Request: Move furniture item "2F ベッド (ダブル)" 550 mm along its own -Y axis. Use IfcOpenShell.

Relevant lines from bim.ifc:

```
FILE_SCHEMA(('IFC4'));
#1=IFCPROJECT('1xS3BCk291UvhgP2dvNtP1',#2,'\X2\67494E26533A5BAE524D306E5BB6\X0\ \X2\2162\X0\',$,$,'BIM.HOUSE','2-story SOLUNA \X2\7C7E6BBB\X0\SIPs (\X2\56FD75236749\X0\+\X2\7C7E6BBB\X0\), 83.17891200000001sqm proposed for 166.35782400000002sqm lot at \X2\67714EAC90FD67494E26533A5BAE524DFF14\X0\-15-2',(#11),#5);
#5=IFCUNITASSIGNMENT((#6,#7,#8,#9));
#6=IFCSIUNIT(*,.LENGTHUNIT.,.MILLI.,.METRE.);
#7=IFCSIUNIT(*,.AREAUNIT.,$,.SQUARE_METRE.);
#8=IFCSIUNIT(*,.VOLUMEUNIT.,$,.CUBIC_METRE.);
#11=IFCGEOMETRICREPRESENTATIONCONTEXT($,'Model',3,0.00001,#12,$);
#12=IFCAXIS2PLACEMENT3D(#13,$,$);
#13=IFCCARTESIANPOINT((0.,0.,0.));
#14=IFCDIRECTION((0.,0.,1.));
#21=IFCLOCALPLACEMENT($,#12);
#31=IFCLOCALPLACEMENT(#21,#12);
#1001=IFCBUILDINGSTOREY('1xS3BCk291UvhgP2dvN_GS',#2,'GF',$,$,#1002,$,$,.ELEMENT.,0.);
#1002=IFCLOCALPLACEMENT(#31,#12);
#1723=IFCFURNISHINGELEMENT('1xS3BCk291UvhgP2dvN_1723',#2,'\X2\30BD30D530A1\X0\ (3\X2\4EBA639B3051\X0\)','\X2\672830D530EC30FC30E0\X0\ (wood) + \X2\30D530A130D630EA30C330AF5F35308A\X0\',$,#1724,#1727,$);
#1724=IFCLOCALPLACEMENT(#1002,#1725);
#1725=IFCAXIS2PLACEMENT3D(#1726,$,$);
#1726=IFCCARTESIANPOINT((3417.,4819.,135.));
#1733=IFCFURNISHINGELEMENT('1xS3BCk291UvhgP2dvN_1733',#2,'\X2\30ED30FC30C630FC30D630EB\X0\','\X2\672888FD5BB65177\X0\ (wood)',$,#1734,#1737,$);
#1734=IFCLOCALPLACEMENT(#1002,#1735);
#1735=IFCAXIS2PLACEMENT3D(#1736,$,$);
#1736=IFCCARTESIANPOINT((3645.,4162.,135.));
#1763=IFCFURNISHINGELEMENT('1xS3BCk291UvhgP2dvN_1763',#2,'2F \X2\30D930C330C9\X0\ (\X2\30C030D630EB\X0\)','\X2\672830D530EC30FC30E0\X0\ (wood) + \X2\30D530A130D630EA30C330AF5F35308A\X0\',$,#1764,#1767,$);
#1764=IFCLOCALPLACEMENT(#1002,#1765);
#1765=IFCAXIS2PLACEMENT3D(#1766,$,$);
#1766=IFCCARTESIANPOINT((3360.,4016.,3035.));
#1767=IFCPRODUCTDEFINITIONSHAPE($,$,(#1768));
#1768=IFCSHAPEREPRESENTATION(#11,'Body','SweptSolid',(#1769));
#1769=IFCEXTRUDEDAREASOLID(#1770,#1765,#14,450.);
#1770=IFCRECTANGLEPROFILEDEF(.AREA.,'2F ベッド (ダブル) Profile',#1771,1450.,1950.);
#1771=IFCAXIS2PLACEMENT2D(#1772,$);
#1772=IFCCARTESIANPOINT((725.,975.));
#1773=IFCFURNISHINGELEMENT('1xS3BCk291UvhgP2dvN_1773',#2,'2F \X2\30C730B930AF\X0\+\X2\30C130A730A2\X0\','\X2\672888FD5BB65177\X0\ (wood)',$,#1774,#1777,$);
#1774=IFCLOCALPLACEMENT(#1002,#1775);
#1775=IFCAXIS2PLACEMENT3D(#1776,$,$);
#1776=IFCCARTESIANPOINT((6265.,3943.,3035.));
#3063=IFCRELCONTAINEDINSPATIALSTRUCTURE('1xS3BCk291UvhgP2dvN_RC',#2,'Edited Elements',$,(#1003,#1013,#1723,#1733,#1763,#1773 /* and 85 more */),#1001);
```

```python
import ifcopenshell
import ifcopenshell.api.geometry
import ifcopenshell.util.placement

model = ifcopenshell.open("bim.ifc")

item = model.by_guid("1xS3BCk291UvhgP2dvN_1763")
matrix = ifcopenshell.util.placement.get_local_placement(item.ObjectPlacement)
matrix[:3, 3] -= matrix[:3, 1] * 550.0
ifcopenshell.api.geometry.edit_object_placement(model, product=item, matrix=matrix, is_si=False)

print(ifcopenshell.util.placement.get_local_placement(item.ObjectPlacement).round(3) + 0.0)

model.write("bim_rev.ifc")
```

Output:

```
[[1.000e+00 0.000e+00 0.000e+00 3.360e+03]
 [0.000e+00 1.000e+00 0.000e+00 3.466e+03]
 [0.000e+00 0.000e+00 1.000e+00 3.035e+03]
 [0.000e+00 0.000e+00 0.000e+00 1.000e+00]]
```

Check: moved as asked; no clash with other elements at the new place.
